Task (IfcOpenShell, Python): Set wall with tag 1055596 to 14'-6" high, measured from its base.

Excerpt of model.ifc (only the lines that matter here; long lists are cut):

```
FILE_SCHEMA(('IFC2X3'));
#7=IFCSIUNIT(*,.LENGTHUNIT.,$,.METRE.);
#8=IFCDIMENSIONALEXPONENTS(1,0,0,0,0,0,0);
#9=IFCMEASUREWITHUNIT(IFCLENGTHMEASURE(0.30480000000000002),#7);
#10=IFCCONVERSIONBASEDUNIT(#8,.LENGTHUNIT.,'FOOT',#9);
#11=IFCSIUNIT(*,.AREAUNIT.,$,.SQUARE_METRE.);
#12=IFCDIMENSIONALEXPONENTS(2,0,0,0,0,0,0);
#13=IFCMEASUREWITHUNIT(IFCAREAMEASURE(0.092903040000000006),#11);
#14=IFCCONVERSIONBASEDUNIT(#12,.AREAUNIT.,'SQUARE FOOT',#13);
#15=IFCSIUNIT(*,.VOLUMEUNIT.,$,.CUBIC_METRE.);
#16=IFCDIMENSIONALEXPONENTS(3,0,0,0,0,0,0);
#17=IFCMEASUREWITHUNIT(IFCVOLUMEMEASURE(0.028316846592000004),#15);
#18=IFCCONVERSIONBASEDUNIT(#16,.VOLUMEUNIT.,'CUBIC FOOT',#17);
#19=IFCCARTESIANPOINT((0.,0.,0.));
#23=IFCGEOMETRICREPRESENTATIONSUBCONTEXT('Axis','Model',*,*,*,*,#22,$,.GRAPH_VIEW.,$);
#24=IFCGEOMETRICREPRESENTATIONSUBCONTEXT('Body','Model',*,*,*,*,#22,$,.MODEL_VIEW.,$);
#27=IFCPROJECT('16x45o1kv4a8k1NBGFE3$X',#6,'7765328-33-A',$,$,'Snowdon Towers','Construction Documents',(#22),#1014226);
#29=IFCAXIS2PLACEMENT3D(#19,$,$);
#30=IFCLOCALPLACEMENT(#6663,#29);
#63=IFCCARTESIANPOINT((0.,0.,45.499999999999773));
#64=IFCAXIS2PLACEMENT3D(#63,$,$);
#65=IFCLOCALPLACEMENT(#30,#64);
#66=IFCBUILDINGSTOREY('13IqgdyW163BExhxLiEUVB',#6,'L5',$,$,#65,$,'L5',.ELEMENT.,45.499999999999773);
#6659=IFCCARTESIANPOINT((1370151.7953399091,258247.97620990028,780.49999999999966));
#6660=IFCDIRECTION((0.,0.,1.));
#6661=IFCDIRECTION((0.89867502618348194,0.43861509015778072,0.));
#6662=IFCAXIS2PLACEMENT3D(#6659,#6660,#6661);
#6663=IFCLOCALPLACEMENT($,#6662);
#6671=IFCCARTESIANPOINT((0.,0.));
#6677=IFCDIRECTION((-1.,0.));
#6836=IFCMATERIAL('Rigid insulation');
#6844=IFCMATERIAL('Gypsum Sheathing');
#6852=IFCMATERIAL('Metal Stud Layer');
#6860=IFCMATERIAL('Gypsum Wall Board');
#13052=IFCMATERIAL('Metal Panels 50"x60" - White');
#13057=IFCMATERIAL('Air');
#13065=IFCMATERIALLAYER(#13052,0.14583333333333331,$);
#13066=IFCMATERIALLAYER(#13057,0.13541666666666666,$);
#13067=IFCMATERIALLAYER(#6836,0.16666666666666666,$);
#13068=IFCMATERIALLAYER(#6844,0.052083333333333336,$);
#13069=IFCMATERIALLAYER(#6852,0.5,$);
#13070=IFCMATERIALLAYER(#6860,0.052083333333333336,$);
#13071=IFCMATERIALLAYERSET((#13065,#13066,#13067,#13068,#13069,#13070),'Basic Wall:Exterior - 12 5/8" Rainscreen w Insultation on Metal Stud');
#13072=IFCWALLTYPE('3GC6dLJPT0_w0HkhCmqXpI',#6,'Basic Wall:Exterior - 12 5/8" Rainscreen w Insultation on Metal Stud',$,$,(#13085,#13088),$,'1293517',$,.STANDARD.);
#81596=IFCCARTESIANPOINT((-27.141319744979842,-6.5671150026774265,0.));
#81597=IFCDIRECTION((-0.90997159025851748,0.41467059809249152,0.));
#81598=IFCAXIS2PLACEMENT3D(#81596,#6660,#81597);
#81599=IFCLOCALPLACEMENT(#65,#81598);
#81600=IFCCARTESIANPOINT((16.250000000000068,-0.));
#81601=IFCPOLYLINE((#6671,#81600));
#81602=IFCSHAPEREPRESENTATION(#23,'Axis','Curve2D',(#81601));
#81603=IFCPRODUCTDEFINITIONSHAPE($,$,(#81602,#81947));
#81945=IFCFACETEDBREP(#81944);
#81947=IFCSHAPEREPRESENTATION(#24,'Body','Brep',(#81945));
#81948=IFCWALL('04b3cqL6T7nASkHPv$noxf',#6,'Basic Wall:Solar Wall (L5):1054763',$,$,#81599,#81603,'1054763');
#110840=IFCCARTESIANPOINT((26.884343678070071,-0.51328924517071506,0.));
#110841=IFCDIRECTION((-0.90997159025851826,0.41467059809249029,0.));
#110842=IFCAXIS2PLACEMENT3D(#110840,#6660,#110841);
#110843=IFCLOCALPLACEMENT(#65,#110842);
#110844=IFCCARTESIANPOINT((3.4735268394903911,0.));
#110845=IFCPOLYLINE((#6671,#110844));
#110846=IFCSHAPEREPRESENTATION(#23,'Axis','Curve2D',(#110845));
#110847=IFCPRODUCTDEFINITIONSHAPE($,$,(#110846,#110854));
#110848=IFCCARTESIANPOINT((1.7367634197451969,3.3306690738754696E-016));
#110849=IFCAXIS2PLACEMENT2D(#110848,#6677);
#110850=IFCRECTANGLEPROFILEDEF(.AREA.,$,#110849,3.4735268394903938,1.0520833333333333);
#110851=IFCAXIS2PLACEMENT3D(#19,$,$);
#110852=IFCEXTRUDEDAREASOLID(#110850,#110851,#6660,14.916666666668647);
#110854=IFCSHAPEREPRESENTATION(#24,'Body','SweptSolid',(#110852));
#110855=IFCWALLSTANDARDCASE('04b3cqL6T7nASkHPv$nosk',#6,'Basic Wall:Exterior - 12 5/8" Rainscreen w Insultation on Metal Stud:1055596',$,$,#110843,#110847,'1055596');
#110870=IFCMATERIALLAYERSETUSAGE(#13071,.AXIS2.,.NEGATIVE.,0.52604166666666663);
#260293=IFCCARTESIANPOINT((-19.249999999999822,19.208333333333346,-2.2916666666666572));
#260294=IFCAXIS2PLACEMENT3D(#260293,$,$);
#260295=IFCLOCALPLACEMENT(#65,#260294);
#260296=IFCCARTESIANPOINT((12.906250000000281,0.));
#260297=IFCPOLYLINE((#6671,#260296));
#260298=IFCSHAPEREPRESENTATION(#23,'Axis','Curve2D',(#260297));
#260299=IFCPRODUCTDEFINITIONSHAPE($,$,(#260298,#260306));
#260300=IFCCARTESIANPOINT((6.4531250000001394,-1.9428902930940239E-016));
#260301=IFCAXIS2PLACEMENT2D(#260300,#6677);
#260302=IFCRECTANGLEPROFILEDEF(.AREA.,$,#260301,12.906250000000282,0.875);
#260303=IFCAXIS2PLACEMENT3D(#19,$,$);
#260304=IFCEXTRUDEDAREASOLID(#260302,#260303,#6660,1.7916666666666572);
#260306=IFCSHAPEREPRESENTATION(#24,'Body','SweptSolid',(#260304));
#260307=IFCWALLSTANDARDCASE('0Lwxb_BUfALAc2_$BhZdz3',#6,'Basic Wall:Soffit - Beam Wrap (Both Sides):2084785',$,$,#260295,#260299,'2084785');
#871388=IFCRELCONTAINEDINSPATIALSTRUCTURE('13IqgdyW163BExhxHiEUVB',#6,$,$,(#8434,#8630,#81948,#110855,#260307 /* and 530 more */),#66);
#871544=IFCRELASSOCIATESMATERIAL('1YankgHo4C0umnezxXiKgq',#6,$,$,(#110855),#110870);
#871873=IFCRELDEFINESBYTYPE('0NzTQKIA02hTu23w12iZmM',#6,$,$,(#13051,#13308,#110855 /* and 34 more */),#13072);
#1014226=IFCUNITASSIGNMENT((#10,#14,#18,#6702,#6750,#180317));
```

```python
import ifcopenshell
import ifcopenshell.geom
import ifcopenshell.util.representation
import ifcopenshell.util.shape
import ifcopenshell.util.unit

model = ifcopenshell.open("model.ifc")
unit_scale = ifcopenshell.util.unit.calculate_unit_scale(model)
settings = ifcopenshell.geom.settings()


def volume(element):
    """Net volume in cubic metres, openings subtracted."""
    shape = ifcopenshell.geom.create_shape(settings, element)
    return ifcopenshell.util.shape.get_volume(shape.geometry)


wall = model.by_guid("04b3cqL6T7nASkHPv$nosk")
before = volume(wall)

body = ifcopenshell.util.representation.get_representation(wall, "Model", "Body")
solid = body.Items[0]
old_height = solid.Depth
solid.Depth = 174 * 0.0254 / unit_scale
after = volume(wall)

print(f"height {old_height:g} -> {solid.Depth:g}, volume {before:.3f} -> {after:.3f} m3")

model.write("model_updated.ifc")
```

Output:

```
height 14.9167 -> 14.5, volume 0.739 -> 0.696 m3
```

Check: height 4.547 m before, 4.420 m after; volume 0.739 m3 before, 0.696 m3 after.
